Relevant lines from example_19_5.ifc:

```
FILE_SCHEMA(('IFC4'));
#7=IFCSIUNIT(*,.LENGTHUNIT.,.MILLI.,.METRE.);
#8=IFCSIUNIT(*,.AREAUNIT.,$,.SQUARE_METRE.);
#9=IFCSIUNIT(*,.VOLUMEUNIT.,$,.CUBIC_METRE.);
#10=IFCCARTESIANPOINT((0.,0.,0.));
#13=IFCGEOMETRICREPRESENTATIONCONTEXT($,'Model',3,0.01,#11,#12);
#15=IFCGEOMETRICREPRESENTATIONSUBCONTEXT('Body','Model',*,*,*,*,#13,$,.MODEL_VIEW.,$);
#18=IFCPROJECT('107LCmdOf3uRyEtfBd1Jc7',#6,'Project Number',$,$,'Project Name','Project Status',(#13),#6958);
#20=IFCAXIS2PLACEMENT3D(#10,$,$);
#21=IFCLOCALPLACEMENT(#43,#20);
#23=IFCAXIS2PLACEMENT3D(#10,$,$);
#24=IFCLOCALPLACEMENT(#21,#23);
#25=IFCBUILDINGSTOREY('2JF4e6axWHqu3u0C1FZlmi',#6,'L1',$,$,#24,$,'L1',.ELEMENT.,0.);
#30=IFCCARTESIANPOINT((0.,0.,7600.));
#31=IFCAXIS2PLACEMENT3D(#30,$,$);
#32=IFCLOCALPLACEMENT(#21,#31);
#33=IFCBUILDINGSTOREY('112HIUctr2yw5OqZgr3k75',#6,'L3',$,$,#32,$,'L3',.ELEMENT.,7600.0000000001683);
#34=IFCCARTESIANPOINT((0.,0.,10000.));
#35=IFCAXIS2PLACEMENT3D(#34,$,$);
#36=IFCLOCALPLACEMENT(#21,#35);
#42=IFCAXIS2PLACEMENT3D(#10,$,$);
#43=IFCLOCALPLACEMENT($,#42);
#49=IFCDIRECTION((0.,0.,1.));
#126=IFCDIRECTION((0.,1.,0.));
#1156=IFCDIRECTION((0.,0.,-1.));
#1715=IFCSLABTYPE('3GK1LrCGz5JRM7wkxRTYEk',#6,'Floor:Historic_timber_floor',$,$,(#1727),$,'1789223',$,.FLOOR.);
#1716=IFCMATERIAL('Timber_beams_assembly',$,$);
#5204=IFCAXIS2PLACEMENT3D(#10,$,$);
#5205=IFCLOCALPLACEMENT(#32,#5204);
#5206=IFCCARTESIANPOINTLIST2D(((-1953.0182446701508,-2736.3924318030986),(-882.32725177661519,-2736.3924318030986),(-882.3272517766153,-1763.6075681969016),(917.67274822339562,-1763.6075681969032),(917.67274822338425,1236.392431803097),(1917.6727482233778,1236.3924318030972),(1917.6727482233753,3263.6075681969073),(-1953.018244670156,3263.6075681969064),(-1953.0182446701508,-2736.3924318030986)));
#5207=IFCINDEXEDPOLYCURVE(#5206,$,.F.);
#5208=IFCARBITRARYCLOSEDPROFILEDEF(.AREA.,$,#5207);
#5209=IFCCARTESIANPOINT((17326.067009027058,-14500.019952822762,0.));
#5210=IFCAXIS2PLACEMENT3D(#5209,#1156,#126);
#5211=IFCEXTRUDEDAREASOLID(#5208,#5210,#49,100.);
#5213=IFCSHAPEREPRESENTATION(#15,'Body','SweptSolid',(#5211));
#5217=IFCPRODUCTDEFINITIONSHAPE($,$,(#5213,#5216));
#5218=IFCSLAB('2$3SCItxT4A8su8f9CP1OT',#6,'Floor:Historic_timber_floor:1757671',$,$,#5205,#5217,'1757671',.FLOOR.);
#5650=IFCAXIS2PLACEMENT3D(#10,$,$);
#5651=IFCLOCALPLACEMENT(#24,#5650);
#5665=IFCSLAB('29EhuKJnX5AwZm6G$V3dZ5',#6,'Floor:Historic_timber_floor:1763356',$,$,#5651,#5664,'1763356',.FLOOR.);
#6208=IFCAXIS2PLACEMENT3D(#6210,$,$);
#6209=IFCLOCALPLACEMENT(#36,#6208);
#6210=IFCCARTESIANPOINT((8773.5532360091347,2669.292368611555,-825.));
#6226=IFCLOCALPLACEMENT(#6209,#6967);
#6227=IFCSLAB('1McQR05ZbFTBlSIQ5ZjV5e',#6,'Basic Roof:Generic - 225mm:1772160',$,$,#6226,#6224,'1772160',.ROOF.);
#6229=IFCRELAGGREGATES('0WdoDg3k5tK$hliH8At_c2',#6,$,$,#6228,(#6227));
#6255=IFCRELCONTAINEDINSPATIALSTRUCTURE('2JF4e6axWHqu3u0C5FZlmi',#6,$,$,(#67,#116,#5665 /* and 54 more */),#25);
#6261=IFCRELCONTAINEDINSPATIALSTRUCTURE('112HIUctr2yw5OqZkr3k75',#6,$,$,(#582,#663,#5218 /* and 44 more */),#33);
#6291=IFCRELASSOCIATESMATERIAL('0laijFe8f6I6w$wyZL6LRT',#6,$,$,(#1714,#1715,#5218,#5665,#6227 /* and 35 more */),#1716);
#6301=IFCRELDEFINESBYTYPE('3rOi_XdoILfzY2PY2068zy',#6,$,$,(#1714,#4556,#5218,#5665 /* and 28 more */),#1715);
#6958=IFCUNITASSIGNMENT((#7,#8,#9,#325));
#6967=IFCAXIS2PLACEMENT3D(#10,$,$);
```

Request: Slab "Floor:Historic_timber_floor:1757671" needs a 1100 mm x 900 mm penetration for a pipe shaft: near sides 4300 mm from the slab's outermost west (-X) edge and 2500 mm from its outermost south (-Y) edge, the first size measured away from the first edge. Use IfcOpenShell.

```python
import numpy as np
import ifcopenshell
import ifcopenshell.api.feature
import ifcopenshell.api.geometry
import ifcopenshell.api.root
import ifcopenshell.geom
import ifcopenshell.util.placement
import ifcopenshell.util.representation
import ifcopenshell.util.shape
import ifcopenshell.util.unit

model = ifcopenshell.open("example_19_5.ifc")
unit_scale = ifcopenshell.util.unit.calculate_unit_scale(model)
settings = ifcopenshell.geom.settings()


def volume(element):
    """Net volume in cubic metres, openings subtracted."""
    shape = ifcopenshell.geom.create_shape(settings, element)
    return ifcopenshell.util.shape.get_volume(shape.geometry)


slab = model.by_guid("2$3SCItxT4A8su8f9CP1OT")
before = volume(slab)

# Extent in the slab's own axes, in metres. The edges named are its -X and -Y sides.
slab_shape = ifcopenshell.geom.create_shape(settings, slab)
vertices = ifcopenshell.util.shape.get_vertices(slab_shape.geometry)
x_min, y_min, bottom = vertices.min(axis=0)
top = vertices[:, 2].max()

opening = ifcopenshell.api.root.create_entity(model, ifc_class="IfcOpeningElement", name="Pipe shaft opening", predefined_type="OPENING")
context = ifcopenshell.util.representation.get_context(model, "Model", "Body", "MODEL_VIEW")
width, depth = 1.1, 0.9
outline = [(0.0, 0.0), (width, 0.0), (width, depth), (0.0, depth), (0.0, 0.0)]
# Overshoot both faces by 50 mm so the cut is clean.
shape = ifcopenshell.api.geometry.add_slab_representation(
    model, context=context, depth=top - bottom + 0.1, polyline=outline
)
ifcopenshell.api.geometry.assign_representation(model, product=opening, representation=shape)

matrix = ifcopenshell.util.placement.get_local_placement(slab.ObjectPlacement)
matrix[:, 3] = matrix @ np.append(np.array([x_min + 4.3, y_min + 2.5, bottom - 0.05]) / unit_scale, 1.0)
ifcopenshell.api.geometry.edit_object_placement(model, product=opening, matrix=matrix, is_si=False)
ifcopenshell.api.feature.add_feature(model, feature=opening, element=slab)

after = volume(slab)

print(f"slab volume {before:.3f} -> {after:.3f} m3")

model.write("example_19_5_rev.ifc")
```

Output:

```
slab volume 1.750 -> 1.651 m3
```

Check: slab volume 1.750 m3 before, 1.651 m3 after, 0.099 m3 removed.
